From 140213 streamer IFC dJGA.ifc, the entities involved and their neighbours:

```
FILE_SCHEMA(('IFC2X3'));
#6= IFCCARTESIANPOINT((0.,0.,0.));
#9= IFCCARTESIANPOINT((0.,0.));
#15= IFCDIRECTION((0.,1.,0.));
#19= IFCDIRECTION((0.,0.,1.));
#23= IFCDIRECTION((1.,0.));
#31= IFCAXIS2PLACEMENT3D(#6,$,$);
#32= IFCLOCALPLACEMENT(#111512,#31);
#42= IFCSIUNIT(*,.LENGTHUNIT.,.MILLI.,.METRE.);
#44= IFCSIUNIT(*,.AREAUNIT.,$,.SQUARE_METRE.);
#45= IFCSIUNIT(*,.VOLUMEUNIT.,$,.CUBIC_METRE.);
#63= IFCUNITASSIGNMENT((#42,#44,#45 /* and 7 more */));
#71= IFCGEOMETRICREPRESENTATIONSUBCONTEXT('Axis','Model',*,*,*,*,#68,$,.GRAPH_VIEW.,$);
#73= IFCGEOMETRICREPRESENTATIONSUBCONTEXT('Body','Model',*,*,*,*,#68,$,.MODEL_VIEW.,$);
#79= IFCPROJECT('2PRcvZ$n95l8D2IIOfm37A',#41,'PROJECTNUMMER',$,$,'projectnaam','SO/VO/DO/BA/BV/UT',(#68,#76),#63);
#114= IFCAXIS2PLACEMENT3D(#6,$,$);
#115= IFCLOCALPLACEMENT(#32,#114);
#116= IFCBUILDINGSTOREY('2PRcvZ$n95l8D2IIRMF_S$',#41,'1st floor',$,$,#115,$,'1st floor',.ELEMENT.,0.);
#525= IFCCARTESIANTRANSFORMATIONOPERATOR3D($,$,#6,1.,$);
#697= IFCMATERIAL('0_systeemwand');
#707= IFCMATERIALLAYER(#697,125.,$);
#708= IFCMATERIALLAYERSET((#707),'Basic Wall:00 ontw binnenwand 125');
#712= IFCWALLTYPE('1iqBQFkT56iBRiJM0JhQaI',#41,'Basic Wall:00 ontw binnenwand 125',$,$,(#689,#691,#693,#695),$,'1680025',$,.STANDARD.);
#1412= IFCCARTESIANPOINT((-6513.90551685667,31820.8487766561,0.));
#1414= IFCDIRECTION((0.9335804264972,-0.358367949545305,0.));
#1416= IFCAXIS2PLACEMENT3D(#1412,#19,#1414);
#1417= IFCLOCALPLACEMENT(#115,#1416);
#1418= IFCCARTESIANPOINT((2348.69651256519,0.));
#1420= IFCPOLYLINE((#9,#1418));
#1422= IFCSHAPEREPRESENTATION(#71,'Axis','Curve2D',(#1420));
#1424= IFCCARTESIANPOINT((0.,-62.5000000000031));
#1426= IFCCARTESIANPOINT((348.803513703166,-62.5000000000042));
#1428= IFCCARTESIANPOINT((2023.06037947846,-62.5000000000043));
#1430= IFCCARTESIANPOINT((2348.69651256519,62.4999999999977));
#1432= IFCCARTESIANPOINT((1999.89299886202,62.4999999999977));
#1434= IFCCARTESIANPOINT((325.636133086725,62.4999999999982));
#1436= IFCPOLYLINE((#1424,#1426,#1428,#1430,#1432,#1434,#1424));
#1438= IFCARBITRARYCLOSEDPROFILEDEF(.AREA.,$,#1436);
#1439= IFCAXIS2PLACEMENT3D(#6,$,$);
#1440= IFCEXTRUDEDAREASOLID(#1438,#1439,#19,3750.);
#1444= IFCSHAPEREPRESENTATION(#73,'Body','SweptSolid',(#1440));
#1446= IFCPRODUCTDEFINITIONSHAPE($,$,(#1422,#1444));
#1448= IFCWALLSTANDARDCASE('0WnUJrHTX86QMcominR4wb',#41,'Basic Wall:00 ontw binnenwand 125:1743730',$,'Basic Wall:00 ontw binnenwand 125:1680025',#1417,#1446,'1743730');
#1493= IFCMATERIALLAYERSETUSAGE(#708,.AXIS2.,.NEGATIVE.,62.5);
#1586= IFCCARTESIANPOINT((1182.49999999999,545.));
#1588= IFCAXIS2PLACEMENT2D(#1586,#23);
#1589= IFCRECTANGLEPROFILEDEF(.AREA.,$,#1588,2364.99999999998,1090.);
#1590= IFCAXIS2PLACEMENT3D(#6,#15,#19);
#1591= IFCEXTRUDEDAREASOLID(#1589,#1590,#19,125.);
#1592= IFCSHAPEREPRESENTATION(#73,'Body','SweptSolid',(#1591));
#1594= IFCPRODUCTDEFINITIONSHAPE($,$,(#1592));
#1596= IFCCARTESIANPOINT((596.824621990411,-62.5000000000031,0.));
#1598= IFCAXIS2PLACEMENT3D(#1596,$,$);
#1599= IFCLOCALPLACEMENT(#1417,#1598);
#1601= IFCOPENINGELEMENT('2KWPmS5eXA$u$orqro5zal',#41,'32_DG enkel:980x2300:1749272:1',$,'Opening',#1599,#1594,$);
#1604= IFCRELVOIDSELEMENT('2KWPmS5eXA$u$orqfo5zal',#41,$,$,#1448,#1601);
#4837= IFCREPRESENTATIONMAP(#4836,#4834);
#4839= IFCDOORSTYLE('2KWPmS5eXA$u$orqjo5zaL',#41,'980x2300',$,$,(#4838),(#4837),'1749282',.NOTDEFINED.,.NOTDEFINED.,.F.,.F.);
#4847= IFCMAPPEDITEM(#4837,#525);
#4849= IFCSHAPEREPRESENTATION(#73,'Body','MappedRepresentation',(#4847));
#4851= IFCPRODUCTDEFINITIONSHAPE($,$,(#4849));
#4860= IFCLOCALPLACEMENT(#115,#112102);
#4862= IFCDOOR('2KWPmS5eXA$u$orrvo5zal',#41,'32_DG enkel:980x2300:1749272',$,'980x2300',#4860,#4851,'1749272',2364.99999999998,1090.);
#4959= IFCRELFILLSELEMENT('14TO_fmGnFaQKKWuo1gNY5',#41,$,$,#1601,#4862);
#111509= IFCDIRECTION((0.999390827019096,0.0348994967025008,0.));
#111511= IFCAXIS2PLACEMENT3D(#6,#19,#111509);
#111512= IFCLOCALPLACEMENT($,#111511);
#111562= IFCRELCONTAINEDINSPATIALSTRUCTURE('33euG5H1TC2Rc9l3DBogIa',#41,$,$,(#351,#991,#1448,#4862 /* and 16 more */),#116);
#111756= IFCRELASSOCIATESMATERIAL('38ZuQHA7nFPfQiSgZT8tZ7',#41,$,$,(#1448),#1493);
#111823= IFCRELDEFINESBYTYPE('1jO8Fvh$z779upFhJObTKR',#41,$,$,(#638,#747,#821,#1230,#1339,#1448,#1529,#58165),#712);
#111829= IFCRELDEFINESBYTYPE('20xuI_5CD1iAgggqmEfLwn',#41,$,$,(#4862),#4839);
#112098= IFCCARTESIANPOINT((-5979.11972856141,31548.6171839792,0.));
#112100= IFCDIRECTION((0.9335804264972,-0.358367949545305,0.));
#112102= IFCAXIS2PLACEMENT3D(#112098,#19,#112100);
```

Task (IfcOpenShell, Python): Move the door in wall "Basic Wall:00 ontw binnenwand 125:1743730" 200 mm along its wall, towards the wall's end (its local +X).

```python
import ifcopenshell
import ifcopenshell.api.geometry
import ifcopenshell.util.placement
import ifcopenshell.util.unit

model = ifcopenshell.open("140213 streamer IFC dJGA.ifc")
unit_scale = ifcopenshell.util.unit.calculate_unit_scale(model)

door = model.by_id(4862)
opening = door.FillsVoids[0].RelatingOpeningElement
wall = opening.VoidsElements[0].RelatingBuildingElement

wall_matrix = ifcopenshell.util.placement.get_local_placement(wall.ObjectPlacement)
shift = wall_matrix[:3, 0] * 0.2 / unit_scale
before = ifcopenshell.util.placement.get_local_placement(door.ObjectPlacement)[:3, 3].copy()

# The door is not placed relative to its opening, so move both.
for product in (opening, door):
    matrix = ifcopenshell.util.placement.get_local_placement(product.ObjectPlacement)
    matrix[:3, 3] += shift
    ifcopenshell.api.geometry.edit_object_placement(model, product=product, matrix=matrix, is_si=False)

after = ifcopenshell.util.placement.get_local_placement(door.ObjectPlacement)[:3, 3]
print("door moved by", (after - before).round(3) + 0.0)

model.write("140213 streamer IFC dJGA_rev.ifc")
```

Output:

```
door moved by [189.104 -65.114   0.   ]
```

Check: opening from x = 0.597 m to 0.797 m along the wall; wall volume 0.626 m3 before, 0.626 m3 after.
